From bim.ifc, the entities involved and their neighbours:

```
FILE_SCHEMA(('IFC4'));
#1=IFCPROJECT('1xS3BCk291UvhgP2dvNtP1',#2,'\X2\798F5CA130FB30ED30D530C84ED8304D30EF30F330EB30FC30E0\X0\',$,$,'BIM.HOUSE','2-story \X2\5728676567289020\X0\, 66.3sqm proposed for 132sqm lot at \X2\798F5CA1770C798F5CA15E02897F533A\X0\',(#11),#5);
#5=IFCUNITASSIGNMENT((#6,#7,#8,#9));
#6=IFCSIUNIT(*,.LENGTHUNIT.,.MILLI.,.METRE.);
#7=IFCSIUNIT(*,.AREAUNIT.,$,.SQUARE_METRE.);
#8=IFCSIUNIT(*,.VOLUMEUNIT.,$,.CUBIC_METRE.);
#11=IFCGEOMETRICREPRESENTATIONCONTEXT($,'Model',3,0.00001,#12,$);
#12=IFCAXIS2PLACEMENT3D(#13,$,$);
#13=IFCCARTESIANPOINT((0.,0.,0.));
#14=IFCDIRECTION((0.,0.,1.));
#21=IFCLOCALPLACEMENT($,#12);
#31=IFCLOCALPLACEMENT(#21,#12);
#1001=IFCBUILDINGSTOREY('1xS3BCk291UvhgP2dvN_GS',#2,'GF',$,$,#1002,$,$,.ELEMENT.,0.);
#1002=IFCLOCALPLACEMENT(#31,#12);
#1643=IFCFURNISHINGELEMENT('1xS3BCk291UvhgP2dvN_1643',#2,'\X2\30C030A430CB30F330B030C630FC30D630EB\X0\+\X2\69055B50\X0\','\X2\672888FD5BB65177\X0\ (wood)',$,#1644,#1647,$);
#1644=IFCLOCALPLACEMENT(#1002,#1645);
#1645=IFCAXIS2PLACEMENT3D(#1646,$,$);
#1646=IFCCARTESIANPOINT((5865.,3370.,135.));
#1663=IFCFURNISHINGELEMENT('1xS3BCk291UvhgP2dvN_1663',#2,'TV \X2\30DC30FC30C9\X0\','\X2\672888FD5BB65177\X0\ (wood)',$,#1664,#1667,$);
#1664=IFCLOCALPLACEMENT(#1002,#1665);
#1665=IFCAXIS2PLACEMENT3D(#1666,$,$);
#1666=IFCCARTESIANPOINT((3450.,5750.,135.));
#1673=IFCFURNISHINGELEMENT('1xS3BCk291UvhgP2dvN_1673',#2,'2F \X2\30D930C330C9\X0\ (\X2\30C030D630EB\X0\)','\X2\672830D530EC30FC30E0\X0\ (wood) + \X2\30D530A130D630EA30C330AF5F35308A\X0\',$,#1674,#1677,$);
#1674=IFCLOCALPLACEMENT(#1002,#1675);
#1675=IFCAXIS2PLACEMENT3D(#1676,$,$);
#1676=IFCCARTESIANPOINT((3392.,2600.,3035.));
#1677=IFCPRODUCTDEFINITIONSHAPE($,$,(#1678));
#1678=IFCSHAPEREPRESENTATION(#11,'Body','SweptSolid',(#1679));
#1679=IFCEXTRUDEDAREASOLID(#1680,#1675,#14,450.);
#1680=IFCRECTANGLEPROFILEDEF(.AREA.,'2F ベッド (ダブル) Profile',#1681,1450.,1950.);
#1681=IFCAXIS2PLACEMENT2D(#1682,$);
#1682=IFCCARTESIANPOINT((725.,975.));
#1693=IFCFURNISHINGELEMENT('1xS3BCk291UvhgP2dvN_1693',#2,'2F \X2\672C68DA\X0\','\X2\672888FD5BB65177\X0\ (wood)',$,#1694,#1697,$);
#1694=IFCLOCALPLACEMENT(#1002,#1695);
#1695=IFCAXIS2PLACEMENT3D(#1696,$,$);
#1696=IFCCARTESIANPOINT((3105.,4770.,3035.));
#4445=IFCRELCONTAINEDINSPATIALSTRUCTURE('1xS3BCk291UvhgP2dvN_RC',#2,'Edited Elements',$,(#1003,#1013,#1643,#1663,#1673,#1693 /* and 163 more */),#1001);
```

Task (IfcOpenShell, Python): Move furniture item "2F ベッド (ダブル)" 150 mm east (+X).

```python
import ifcopenshell
import ifcopenshell.api.geometry
import ifcopenshell.util.placement

model = ifcopenshell.open("bim.ifc")

item = model.by_guid("1xS3BCk291UvhgP2dvN_1673")
matrix = ifcopenshell.util.placement.get_local_placement(item.ObjectPlacement)
matrix[0, 3] += 150.0
ifcopenshell.api.geometry.edit_object_placement(model, product=item, matrix=matrix, is_si=False)

print(ifcopenshell.util.placement.get_local_placement(item.ObjectPlacement).round(3) + 0.0)

model.write("bim_v2.ifc")
```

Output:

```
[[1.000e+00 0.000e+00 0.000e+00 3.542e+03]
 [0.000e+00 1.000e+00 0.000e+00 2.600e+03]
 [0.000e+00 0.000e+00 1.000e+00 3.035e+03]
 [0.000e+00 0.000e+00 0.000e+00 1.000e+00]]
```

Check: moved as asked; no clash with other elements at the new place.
